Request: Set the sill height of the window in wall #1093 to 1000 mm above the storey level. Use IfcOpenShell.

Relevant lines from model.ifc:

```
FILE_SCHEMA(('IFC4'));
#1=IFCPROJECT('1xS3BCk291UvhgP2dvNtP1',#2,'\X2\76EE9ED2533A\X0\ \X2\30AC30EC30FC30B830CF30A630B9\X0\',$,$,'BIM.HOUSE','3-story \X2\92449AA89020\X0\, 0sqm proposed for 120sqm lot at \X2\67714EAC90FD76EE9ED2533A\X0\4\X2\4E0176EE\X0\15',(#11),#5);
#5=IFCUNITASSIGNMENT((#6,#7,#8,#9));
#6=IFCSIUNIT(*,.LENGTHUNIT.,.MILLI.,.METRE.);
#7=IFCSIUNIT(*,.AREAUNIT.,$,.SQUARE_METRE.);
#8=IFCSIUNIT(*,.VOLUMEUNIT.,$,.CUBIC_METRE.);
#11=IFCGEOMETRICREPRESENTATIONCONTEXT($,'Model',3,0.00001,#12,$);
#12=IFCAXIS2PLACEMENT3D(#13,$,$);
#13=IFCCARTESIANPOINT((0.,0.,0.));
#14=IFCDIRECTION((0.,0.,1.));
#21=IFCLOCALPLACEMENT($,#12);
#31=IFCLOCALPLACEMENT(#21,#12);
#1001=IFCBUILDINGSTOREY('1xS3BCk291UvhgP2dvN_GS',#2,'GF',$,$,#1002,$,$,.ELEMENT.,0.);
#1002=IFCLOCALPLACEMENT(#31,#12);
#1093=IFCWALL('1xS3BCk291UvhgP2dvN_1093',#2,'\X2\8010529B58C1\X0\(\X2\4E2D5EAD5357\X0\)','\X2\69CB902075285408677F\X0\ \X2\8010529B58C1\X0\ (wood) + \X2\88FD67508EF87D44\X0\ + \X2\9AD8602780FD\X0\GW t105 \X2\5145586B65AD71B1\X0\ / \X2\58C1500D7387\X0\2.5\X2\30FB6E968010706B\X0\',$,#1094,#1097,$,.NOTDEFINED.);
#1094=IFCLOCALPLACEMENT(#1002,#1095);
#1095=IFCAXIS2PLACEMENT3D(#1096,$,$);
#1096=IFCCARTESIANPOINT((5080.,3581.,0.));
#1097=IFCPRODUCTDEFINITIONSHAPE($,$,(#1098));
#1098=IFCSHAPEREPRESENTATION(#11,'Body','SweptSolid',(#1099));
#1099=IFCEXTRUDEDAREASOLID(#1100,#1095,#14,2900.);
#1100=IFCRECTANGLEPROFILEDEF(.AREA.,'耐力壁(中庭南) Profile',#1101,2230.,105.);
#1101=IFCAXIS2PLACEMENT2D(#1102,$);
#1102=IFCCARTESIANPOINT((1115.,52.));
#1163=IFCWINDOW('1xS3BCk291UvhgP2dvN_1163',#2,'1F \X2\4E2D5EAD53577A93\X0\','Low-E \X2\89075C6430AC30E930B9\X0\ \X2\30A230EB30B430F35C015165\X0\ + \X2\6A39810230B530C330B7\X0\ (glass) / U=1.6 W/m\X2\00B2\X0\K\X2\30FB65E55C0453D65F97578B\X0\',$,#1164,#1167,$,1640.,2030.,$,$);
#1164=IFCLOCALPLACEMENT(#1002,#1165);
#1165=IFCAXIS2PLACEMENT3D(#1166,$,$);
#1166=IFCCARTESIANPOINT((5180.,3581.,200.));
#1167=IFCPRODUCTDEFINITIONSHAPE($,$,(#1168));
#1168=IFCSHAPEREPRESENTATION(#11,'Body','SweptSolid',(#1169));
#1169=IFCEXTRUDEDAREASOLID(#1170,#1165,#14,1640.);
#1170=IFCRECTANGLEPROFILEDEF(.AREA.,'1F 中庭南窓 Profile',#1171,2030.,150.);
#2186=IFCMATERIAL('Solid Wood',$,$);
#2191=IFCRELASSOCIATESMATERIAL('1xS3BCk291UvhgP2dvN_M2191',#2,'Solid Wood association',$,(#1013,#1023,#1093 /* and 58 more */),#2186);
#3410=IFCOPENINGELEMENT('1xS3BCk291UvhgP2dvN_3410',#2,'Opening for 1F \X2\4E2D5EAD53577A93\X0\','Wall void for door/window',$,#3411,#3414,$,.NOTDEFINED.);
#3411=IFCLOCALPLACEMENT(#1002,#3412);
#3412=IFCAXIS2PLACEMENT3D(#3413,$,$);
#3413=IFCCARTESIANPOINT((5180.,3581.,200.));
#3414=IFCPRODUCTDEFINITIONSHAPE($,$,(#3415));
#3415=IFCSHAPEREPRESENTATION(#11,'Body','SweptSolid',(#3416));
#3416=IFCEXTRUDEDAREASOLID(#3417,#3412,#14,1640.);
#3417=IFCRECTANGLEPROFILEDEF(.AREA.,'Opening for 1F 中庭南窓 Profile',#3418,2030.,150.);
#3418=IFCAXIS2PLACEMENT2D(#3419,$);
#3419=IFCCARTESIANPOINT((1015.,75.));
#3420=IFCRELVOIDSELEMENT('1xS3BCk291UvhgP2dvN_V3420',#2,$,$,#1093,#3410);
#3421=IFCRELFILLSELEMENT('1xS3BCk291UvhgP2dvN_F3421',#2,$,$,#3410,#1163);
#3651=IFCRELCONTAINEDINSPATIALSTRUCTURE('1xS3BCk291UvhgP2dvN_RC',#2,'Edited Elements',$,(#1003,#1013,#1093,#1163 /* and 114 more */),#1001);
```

```python
import numpy as np
import ifcopenshell
import ifcopenshell.api.geometry
import ifcopenshell.geom
import ifcopenshell.util.element
import ifcopenshell.util.placement
import ifcopenshell.util.shape
import ifcopenshell.util.unit

model = ifcopenshell.open("model.ifc")
unit_scale = ifcopenshell.util.unit.calculate_unit_scale(model)

window = model.by_id(1163)
opening = window.FillsVoids[0].RelatingOpeningElement
storey = ifcopenshell.util.element.get_container(window, ifc_class="IfcBuildingStorey")
level = ifcopenshell.util.placement.get_local_placement(storey.ObjectPlacement)[2, 3]

# The opening's origin need not be at the sill, so measure its lowest point.
shape = ifcopenshell.geom.create_shape(ifcopenshell.geom.settings(), opening)
bottom = ifcopenshell.util.shape.get_shape_bottom_elevation(shape, shape.geometry) / unit_scale
dz = level + 1000.0 - bottom

shift = np.array([0.0, 0.0, dz])
# The window is not placed relative to its opening, so move both.
for product in (opening, window):
    matrix = ifcopenshell.util.placement.get_local_placement(product.ObjectPlacement)
    matrix[:3, 3] += shift
    ifcopenshell.api.geometry.edit_object_placement(model, product=product, matrix=matrix, is_si=False)

print(f"moved by {dz * unit_scale:+.3f} m")

model.write("model_edited.ifc")
```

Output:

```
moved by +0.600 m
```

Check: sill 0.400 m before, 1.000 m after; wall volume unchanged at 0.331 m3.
